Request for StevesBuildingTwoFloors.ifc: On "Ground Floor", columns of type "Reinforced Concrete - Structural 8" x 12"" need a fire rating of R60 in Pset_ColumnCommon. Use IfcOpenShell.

First a look at what the model holds.

```python
import ifcopenshell
import ifcopenshell.util.element

model = ifcopenshell.open("StevesBuildingTwoFloors.ifc")
print(model.schema)
storey = next(s for s in model.by_type("IfcBuildingStorey") if s.Name == "Ground Floor")
columns = [e for e in ifcopenshell.util.element.get_decomposition(storey) if e.is_a("IfcColumn")]
seen = {}
for e in columns:
    element_type = ifcopenshell.util.element.get_type(e)
    key = (element_type.Name if element_type != e and element_type else None, ifcopenshell.util.element.get_pset(e, "Pset_ColumnCommon", "FireRating"))
    seen[key] = seen.get(key, 0) + 1
for (name, value), count in sorted(seen.items(), key=str):
    print(count, "x", name, "|", value)
```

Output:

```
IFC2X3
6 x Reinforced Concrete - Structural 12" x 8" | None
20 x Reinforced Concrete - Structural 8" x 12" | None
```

```python
import ifcopenshell
import ifcopenshell.api.pset
import ifcopenshell.util.element

model = ifcopenshell.open("StevesBuildingTwoFloors.ifc")

storey = next(s for s in model.by_type("IfcBuildingStorey") if s.Name == "Ground Floor")
columns = [e for e in ifcopenshell.util.element.get_decomposition(storey) if e.is_a("IfcColumn")]

count = 0
for e in columns:
    element_type = ifcopenshell.util.element.get_type(e)
    if element_type in (None, e) or element_type.Name != 'Reinforced Concrete - Structural 8" x 12"':
        continue
    # add_pset returns the element's existing set when there is one.
    pset = ifcopenshell.api.pset.add_pset(model, product=e, name="Pset_ColumnCommon")
    ifcopenshell.api.pset.edit_pset(model, pset=pset, properties={"FireRating": "R60"})
    count += 1

print(count, "columns updated")

model.write("StevesBuildingTwoFloors_edited.ifc")
```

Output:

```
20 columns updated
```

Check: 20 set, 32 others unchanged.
